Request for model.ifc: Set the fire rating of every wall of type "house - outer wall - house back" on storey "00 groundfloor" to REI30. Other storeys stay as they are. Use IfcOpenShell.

First a look at what the model holds.

```python
import ifcopenshell
import ifcopenshell.util.element

model = ifcopenshell.open("model.ifc")
print(model.schema)
storey = next(s for s in model.by_type("IfcBuildingStorey") if s.Name == "00 groundfloor")
walls = [e for e in ifcopenshell.util.element.get_decomposition(storey) if e.is_a("IfcWall")]
seen = {}
for e in walls:
    element_type = ifcopenshell.util.element.get_type(e)
    key = (element_type.Name if element_type != e and element_type else None, ifcopenshell.util.element.get_pset(e, "Pset_WallCommon", "FireRating"))
    seen[key] = seen.get(key, 0) + 1
for (name, value), count in sorted(seen.items(), key=str):
    print(count, "x", name, "|", value)
```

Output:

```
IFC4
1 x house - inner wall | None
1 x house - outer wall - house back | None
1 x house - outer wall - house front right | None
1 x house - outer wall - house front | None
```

```python
import ifcopenshell
import ifcopenshell.api.pset
import ifcopenshell.util.element

model = ifcopenshell.open("model.ifc")

storey = next(s for s in model.by_type("IfcBuildingStorey") if s.Name == "00 groundfloor")
walls = [e for e in ifcopenshell.util.element.get_decomposition(storey) if e.is_a("IfcWall")]

count = 0
for e in walls:
    element_type = ifcopenshell.util.element.get_type(e)
    if element_type in (None, e) or element_type.Name != "house - outer wall - house back":
        continue
    # add_pset returns the element's existing set when there is one.
    pset = ifcopenshell.api.pset.add_pset(model, product=e, name="Pset_WallCommon")
    ifcopenshell.api.pset.edit_pset(model, pset=pset, properties={"FireRating": "REI30"})
    count += 1

print(count, "walls updated")

model.write("model_rev.ifc")
```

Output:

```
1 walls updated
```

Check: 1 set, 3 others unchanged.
